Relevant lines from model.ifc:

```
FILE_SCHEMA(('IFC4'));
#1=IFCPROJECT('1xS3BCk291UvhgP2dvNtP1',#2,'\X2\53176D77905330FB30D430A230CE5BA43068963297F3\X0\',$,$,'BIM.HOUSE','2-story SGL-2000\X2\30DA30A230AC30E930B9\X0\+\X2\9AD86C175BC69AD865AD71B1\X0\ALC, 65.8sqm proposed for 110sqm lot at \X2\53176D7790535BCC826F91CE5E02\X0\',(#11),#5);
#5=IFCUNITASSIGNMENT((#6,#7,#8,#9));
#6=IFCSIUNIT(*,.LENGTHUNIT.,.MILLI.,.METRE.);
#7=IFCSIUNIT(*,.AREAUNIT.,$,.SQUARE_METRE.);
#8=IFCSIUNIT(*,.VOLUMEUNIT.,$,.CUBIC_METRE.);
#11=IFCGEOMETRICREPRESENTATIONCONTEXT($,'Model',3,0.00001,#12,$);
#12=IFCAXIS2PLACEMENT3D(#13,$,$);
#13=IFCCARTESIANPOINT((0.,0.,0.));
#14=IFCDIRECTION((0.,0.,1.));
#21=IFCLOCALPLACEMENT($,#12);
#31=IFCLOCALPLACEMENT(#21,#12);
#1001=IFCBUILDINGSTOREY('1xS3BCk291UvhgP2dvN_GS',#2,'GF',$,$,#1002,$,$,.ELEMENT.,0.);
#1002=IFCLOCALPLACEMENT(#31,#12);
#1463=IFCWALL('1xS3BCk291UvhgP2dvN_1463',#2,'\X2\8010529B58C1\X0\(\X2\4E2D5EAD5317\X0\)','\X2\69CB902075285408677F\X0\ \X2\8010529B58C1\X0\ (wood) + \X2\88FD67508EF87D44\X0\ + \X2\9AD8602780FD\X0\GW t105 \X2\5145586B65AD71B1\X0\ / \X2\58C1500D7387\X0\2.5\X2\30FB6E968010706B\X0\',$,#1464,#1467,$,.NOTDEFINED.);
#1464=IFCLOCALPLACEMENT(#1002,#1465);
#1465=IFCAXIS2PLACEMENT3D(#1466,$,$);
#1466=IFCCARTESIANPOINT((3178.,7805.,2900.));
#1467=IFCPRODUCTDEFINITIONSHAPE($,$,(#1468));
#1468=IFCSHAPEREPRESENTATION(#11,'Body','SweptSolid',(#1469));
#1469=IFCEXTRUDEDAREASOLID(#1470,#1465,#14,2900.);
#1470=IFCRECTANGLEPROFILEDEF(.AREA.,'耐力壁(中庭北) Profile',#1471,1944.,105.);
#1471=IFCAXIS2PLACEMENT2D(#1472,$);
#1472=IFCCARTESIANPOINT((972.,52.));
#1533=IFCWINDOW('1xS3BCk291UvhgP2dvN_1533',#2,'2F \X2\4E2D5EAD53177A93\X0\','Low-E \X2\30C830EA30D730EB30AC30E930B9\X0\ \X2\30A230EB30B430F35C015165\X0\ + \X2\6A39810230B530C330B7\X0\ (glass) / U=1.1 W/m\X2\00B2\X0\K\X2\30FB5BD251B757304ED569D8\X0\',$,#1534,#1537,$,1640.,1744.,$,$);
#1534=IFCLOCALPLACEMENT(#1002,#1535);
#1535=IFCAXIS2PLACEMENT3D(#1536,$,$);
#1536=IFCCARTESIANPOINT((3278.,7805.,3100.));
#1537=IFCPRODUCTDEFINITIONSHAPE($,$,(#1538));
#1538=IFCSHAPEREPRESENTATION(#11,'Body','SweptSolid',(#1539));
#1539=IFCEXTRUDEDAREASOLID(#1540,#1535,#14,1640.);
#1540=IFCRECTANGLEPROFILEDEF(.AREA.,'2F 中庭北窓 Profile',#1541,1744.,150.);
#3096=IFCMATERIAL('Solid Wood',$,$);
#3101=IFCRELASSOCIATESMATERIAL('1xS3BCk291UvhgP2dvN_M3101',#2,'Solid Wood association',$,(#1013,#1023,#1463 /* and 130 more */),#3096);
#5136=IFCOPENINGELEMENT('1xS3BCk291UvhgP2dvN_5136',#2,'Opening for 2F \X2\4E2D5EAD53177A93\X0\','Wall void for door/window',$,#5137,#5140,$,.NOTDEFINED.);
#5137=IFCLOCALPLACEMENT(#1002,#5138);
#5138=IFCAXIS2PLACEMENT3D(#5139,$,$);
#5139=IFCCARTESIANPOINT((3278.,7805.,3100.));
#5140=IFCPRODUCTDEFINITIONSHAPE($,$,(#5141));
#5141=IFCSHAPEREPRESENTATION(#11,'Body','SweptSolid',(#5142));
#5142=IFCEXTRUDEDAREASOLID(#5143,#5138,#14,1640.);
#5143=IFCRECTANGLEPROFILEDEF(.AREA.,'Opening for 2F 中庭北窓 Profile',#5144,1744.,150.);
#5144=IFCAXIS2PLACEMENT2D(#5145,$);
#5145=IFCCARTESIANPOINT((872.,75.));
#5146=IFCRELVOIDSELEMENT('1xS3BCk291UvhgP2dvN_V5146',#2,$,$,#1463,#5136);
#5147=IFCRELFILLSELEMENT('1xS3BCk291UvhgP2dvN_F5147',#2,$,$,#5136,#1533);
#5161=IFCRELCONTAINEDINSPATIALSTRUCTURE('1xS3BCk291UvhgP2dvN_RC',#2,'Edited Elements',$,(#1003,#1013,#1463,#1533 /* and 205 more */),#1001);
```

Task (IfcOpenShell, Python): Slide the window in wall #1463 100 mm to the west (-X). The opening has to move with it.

```python
import ifcopenshell
import ifcopenshell.api.geometry
import ifcopenshell.util.placement
import ifcopenshell.util.unit

model = ifcopenshell.open("model.ifc")
unit_scale = ifcopenshell.util.unit.calculate_unit_scale(model)

window = model.by_id(1533)
opening = window.FillsVoids[0].RelatingOpeningElement
wall = opening.VoidsElements[0].RelatingBuildingElement

wall_matrix = ifcopenshell.util.placement.get_local_placement(wall.ObjectPlacement)
shift = wall_matrix[:3, 0] * -0.1 / unit_scale
before = ifcopenshell.util.placement.get_local_placement(window.ObjectPlacement)[:3, 3].copy()

# The window is not placed relative to its opening, so move both.
for product in (opening, window):
    matrix = ifcopenshell.util.placement.get_local_placement(product.ObjectPlacement)
    matrix[:3, 3] += shift
    ifcopenshell.api.geometry.edit_object_placement(model, product=product, matrix=matrix, is_si=False)

after = ifcopenshell.util.placement.get_local_placement(window.ObjectPlacement)[:3, 3]
print("window moved by", (after - before).round(3) + 0.0)

model.write("model_v2.ifc")
```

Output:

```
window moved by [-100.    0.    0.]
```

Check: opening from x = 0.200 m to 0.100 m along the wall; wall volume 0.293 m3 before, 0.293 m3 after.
